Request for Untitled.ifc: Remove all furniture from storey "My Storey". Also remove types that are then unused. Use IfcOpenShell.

First a look at what the model holds.

```python
import ifcopenshell
import ifcopenshell.util.element

model = ifcopenshell.open("Untitled.ifc")
print(model.schema)
storey = next(s for s in model.by_type("IfcBuildingStorey") if s.Name == "My Storey")
furniture = [e for e in ifcopenshell.util.element.get_decomposition(storey) if e.is_a("IfcFurnishingElement")]
seen = {}
for e in furniture:
    element_type = ifcopenshell.util.element.get_type(e)
    name = element_type.Name if element_type not in (None, e) else None
    seen[name] = seen.get(name, 0) + 1
for name, count in sorted(seen.items(), key=str):
    print(count, "x", name)
```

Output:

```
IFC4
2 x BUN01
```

```python
import ifcopenshell
import ifcopenshell.api.root
import ifcopenshell.util.element

model = ifcopenshell.open("Untitled.ifc")

storey = next(s for s in model.by_type("IfcBuildingStorey") if s.Name == "My Storey")
furniture = [e for e in ifcopenshell.util.element.get_decomposition(storey) if e.is_a("IfcFurnishingElement")]
types = {ifcopenshell.util.element.get_type(e) for e in furniture} - {None, *furniture}

for e in furniture:
    ifcopenshell.api.root.remove_product(model, product=e)
print(len(furniture), "removed")

unused = [t for t in types if not ifcopenshell.util.element.get_types(t)]
for t in unused:
    ifcopenshell.api.root.remove_product(model, product=t)
print(len(unused), "unused types removed")

model.write("Untitled_rev.ifc")
```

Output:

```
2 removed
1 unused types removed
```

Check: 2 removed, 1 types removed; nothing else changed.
